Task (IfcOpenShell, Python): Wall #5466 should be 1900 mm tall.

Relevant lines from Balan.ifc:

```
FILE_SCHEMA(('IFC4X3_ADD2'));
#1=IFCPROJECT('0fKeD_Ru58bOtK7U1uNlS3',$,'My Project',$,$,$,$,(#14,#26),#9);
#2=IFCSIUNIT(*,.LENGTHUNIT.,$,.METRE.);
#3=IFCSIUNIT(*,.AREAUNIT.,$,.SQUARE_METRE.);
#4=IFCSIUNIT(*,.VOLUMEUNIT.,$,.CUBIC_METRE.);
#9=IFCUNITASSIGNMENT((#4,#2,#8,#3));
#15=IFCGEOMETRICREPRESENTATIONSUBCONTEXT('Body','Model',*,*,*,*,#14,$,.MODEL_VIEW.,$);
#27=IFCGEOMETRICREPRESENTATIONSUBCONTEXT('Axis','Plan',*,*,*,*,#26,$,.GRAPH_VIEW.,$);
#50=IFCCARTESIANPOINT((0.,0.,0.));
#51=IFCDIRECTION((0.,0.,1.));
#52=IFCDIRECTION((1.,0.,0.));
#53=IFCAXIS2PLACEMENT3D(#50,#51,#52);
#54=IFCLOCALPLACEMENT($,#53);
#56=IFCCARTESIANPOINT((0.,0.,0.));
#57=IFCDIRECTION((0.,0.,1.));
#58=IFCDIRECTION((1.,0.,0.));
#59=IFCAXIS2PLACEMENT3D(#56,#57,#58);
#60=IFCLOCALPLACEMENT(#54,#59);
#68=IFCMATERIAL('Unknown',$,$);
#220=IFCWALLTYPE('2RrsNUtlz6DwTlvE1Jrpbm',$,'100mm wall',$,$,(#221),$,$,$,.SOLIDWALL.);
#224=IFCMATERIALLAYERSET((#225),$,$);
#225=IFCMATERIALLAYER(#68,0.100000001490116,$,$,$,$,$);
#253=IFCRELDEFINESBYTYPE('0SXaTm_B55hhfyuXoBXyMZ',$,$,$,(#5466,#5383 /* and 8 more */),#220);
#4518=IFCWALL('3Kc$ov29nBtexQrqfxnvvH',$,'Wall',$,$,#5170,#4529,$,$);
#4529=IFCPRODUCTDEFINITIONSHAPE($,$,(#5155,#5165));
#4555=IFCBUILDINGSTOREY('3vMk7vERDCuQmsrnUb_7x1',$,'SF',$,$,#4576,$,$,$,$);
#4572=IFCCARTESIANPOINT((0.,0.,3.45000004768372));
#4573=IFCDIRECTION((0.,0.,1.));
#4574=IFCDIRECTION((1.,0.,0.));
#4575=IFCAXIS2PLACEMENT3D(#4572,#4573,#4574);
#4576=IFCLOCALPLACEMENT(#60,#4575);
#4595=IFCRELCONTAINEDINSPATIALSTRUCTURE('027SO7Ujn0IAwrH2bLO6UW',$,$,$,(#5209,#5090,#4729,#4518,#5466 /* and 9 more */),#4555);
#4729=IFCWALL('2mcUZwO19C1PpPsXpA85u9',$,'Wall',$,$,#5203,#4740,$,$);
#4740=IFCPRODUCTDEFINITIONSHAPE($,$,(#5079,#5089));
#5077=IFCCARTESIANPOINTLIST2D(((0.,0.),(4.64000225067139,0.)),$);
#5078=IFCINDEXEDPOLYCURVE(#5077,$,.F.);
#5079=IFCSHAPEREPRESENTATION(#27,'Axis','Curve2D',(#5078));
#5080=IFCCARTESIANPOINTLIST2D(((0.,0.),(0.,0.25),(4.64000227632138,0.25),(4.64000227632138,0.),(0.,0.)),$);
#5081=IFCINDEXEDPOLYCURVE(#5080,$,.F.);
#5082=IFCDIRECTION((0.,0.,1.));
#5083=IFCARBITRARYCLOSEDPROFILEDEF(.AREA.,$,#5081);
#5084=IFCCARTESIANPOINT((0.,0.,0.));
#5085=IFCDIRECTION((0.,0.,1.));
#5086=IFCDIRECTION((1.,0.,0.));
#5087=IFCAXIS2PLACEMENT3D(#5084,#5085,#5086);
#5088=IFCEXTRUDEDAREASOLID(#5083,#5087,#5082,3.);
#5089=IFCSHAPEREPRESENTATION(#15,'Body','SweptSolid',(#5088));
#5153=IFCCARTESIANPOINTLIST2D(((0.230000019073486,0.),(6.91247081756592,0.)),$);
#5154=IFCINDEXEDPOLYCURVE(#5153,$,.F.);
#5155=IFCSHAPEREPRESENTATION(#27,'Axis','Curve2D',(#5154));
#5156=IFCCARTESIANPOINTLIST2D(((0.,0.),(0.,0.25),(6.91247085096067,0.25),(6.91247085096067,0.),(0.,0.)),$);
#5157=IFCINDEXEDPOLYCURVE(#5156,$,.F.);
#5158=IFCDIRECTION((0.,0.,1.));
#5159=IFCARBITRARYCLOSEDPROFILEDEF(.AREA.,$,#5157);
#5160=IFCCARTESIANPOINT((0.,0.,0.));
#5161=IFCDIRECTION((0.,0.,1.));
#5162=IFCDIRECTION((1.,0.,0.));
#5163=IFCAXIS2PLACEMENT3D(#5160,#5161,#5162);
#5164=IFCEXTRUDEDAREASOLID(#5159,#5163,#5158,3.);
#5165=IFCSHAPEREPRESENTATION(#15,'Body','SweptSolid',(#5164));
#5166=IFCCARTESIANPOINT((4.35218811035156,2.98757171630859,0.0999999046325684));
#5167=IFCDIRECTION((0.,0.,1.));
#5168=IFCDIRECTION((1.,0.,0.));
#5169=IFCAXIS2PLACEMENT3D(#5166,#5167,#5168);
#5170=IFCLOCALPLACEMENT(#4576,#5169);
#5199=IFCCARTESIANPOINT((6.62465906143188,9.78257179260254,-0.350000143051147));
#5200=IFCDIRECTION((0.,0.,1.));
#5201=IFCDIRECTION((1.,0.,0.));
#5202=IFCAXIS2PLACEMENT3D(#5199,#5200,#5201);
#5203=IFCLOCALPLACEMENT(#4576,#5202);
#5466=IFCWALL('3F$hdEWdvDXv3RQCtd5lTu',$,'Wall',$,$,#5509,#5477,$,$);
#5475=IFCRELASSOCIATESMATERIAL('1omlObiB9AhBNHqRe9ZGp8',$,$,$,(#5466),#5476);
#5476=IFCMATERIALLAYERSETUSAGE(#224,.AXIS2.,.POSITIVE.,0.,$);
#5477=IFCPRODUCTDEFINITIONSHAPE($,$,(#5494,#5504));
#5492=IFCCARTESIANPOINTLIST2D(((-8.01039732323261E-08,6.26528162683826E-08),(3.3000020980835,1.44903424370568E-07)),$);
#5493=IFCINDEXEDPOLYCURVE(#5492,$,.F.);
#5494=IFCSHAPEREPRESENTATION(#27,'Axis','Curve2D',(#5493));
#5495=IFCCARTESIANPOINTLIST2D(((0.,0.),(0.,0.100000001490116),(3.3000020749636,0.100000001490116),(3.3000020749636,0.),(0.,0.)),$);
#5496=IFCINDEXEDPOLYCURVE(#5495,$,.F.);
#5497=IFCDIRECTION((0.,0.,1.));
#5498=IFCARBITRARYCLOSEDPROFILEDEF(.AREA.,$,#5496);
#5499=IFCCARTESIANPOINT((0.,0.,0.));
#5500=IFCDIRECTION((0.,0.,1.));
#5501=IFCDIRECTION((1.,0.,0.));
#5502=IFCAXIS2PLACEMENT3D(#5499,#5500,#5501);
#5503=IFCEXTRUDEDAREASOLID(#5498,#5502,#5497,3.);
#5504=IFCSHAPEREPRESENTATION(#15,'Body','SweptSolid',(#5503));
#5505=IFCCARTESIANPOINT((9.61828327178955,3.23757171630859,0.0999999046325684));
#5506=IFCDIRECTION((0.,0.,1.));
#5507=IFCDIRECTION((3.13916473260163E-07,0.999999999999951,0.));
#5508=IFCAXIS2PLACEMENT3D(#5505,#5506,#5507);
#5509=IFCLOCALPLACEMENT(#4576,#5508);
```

```python
import ifcopenshell
import ifcopenshell.geom
import ifcopenshell.util.representation
import ifcopenshell.util.shape
import ifcopenshell.util.unit

model = ifcopenshell.open("Balan.ifc")
unit_scale = ifcopenshell.util.unit.calculate_unit_scale(model)
settings = ifcopenshell.geom.settings()


def volume(element):
    """Net volume in cubic metres, openings subtracted."""
    shape = ifcopenshell.geom.create_shape(settings, element)
    return ifcopenshell.util.shape.get_volume(shape.geometry)


wall = model.by_id(5466)
before = volume(wall)

body = ifcopenshell.util.representation.get_representation(wall, "Model", "Body")
solid = body.Items[0]
old_height = solid.Depth
solid.Depth = 1.9 / unit_scale
after = volume(wall)

print(f"height {old_height:g} -> {solid.Depth:g}, volume {before:.3f} -> {after:.3f} m3")

model.write("Balan-out.ifc")
```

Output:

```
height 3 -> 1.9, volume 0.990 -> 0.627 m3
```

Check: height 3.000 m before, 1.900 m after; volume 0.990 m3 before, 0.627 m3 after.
